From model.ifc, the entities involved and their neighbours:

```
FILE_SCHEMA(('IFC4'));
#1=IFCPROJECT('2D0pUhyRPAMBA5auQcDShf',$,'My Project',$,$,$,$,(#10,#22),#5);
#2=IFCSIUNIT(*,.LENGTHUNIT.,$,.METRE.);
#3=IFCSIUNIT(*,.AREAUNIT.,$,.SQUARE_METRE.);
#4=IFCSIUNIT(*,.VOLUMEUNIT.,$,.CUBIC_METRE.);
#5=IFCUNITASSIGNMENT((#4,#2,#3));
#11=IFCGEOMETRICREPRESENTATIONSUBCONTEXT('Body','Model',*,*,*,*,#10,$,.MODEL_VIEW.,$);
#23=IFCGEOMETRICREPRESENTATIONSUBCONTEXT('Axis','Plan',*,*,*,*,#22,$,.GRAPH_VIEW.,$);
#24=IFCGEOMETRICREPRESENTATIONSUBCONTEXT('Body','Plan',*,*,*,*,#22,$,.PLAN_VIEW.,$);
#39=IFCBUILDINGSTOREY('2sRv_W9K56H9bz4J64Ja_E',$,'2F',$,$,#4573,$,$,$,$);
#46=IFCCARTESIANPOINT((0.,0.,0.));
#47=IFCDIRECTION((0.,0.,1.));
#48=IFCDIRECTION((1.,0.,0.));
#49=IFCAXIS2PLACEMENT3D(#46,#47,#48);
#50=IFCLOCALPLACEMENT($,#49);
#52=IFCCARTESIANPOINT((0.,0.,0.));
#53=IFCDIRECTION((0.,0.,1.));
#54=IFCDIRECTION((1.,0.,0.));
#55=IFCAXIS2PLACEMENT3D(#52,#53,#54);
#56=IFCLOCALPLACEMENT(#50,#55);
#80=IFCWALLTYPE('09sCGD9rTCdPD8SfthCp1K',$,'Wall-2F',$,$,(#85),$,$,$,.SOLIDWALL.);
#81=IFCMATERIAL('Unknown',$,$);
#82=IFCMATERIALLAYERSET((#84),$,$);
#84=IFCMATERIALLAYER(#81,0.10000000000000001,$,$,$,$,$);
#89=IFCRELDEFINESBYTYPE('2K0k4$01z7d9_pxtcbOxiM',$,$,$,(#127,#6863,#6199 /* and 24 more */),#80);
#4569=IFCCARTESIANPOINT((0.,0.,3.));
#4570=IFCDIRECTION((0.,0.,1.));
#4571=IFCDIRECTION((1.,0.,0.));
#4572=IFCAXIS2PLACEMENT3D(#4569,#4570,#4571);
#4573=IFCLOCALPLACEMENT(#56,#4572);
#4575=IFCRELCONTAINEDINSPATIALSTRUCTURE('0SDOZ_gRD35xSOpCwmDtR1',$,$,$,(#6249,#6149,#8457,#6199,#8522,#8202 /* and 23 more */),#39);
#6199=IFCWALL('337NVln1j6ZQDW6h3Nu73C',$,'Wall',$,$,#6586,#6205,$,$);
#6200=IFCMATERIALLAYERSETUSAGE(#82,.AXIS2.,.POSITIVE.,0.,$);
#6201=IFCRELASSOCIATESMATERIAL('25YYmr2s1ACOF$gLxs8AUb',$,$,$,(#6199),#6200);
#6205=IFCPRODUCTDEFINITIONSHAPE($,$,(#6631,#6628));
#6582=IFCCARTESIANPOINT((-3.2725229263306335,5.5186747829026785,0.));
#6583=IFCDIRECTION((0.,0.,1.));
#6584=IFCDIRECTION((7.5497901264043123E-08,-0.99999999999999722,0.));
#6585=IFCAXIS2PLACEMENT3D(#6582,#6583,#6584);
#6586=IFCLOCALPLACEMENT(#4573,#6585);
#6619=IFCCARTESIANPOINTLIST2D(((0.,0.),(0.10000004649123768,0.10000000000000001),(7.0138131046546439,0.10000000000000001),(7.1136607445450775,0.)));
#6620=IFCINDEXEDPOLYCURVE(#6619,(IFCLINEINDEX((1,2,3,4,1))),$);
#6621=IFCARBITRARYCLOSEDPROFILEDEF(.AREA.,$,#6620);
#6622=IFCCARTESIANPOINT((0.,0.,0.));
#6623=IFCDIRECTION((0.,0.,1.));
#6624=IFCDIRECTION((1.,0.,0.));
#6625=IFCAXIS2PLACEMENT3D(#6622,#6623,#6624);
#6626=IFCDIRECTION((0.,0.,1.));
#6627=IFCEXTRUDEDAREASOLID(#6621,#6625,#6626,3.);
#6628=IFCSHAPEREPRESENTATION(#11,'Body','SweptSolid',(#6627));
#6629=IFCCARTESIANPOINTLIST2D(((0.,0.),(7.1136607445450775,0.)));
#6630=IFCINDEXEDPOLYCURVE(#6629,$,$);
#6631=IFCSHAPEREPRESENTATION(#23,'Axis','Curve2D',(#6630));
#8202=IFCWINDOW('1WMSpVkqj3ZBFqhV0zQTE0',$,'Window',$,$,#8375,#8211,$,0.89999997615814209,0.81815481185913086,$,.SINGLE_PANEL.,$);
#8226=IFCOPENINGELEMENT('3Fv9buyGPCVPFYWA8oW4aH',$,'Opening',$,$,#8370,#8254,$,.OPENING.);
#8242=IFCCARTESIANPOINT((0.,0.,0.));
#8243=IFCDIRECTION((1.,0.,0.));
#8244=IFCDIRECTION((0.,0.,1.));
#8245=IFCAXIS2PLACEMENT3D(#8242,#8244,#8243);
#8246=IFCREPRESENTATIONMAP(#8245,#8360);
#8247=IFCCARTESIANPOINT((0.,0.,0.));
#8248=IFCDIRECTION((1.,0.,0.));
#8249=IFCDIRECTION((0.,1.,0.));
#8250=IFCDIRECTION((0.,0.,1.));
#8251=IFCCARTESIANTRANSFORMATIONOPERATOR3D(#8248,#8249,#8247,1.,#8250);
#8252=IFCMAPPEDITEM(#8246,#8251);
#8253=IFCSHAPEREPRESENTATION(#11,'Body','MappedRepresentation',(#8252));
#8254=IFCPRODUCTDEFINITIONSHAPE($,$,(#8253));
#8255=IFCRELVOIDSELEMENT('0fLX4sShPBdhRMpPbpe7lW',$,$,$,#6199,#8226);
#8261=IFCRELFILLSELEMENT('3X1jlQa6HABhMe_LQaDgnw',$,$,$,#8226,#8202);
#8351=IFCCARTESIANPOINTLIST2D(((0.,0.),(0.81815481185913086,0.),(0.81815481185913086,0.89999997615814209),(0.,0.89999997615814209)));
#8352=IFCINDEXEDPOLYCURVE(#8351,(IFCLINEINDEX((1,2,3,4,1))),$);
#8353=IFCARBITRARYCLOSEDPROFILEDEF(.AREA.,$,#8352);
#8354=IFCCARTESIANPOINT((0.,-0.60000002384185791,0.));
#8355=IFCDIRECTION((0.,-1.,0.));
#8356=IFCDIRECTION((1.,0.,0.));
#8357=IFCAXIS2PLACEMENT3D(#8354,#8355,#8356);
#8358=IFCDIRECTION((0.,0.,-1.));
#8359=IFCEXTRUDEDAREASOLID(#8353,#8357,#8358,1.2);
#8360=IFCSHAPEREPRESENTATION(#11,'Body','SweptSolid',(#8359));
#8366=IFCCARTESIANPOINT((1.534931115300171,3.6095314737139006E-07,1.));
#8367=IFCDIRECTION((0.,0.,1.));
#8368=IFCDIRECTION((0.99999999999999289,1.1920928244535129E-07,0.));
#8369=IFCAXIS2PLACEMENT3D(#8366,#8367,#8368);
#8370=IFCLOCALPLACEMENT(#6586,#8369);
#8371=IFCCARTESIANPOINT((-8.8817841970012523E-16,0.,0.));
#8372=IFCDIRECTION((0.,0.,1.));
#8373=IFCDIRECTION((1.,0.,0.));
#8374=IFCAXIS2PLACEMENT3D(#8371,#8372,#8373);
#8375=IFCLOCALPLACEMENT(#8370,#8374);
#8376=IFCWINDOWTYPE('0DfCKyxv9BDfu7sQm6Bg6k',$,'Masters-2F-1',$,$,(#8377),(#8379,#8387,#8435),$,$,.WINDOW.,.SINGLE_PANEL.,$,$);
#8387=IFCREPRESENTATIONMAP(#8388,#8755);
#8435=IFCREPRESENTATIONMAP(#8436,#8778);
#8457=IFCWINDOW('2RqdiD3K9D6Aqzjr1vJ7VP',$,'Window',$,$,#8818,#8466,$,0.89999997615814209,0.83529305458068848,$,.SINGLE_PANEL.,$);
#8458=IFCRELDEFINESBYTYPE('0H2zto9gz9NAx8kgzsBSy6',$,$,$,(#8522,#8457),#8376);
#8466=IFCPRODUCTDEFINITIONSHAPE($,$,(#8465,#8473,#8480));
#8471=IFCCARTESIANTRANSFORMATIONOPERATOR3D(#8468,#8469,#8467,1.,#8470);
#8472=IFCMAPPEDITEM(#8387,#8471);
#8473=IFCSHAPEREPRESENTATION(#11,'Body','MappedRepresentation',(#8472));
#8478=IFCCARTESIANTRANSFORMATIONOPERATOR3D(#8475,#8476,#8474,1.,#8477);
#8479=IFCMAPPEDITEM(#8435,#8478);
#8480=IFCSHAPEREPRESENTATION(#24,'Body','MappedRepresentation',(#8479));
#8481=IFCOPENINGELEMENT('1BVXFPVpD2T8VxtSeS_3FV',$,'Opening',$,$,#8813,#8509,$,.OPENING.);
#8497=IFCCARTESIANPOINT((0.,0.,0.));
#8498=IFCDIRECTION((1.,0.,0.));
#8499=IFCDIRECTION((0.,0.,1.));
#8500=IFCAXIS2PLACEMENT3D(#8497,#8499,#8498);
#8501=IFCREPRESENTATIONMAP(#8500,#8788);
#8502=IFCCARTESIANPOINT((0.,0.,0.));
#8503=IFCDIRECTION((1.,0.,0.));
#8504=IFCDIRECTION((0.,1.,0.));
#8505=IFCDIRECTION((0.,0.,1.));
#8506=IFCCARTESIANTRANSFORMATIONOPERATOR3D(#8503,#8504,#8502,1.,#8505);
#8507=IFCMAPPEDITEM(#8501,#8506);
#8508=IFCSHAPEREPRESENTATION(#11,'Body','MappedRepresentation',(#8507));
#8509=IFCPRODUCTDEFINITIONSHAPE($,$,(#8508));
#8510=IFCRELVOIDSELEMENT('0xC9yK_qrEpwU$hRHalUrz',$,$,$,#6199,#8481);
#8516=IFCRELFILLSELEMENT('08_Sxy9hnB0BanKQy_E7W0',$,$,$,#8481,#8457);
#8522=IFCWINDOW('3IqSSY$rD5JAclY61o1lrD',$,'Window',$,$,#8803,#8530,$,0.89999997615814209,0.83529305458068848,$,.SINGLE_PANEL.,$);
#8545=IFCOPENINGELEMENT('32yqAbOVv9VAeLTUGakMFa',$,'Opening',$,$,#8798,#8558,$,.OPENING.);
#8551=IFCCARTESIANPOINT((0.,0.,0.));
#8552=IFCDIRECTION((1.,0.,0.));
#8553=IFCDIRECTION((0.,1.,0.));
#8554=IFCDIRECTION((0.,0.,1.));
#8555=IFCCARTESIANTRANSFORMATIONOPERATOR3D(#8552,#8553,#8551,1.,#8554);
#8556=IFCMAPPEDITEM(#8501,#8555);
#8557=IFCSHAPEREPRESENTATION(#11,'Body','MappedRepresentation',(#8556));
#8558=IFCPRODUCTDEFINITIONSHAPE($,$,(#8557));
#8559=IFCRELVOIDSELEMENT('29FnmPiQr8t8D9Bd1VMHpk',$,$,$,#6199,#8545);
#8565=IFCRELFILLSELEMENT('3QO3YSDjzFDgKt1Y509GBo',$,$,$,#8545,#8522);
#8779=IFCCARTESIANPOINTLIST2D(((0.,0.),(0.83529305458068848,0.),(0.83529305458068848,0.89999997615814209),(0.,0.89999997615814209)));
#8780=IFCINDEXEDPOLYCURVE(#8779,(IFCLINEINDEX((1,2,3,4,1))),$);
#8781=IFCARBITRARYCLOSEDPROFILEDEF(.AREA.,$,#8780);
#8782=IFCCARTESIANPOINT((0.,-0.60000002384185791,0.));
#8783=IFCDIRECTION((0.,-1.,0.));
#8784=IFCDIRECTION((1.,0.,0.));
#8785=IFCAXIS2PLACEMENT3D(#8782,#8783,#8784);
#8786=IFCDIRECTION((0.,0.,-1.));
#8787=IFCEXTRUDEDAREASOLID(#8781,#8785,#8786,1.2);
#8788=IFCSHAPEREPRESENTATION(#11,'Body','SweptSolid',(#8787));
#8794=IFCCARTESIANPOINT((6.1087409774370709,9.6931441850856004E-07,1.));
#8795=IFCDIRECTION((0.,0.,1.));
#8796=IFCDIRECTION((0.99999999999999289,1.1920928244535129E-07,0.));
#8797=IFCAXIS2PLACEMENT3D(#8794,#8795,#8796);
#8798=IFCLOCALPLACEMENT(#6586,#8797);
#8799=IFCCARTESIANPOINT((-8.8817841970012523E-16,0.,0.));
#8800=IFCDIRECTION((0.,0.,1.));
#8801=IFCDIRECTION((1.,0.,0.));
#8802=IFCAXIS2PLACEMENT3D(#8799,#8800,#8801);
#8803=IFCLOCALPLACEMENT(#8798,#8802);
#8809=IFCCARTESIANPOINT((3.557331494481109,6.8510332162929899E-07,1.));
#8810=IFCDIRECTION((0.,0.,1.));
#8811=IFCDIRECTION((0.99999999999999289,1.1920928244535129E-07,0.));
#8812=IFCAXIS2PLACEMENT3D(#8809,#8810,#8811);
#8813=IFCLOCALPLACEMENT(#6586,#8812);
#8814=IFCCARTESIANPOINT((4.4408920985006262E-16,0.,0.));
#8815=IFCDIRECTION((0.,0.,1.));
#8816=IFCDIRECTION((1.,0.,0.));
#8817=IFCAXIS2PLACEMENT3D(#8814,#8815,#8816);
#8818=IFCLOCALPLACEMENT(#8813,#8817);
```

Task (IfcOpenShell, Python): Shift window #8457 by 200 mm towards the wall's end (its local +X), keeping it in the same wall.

```python
import ifcopenshell
import ifcopenshell.api.geometry
import ifcopenshell.util.placement

model = ifcopenshell.open("model.ifc")

window = model.by_guid("2RqdiD3K9D6Aqzjr1vJ7VP")
opening = window.FillsVoids[0].RelatingOpeningElement
wall = opening.VoidsElements[0].RelatingBuildingElement

wall_matrix = ifcopenshell.util.placement.get_local_placement(wall.ObjectPlacement)
shift = wall_matrix[:3, 0] * 0.2
before = ifcopenshell.util.placement.get_local_placement(window.ObjectPlacement)[:3, 3].copy()

# The window is placed relative to its opening, so it follows when the opening moves.
matrix = ifcopenshell.util.placement.get_local_placement(opening.ObjectPlacement)
matrix[:3, 3] += shift
ifcopenshell.api.geometry.edit_object_placement(
    model, product=opening, matrix=matrix, is_si=False, should_transform_children=True
)

after = ifcopenshell.util.placement.get_local_placement(window.ObjectPlacement)[:3, 3]
print("window moved by", (after - before).round(3) + 0.0)

model.write("model_rev.ifc")
```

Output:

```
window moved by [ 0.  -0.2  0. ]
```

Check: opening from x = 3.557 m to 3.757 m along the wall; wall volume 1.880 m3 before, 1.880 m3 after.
